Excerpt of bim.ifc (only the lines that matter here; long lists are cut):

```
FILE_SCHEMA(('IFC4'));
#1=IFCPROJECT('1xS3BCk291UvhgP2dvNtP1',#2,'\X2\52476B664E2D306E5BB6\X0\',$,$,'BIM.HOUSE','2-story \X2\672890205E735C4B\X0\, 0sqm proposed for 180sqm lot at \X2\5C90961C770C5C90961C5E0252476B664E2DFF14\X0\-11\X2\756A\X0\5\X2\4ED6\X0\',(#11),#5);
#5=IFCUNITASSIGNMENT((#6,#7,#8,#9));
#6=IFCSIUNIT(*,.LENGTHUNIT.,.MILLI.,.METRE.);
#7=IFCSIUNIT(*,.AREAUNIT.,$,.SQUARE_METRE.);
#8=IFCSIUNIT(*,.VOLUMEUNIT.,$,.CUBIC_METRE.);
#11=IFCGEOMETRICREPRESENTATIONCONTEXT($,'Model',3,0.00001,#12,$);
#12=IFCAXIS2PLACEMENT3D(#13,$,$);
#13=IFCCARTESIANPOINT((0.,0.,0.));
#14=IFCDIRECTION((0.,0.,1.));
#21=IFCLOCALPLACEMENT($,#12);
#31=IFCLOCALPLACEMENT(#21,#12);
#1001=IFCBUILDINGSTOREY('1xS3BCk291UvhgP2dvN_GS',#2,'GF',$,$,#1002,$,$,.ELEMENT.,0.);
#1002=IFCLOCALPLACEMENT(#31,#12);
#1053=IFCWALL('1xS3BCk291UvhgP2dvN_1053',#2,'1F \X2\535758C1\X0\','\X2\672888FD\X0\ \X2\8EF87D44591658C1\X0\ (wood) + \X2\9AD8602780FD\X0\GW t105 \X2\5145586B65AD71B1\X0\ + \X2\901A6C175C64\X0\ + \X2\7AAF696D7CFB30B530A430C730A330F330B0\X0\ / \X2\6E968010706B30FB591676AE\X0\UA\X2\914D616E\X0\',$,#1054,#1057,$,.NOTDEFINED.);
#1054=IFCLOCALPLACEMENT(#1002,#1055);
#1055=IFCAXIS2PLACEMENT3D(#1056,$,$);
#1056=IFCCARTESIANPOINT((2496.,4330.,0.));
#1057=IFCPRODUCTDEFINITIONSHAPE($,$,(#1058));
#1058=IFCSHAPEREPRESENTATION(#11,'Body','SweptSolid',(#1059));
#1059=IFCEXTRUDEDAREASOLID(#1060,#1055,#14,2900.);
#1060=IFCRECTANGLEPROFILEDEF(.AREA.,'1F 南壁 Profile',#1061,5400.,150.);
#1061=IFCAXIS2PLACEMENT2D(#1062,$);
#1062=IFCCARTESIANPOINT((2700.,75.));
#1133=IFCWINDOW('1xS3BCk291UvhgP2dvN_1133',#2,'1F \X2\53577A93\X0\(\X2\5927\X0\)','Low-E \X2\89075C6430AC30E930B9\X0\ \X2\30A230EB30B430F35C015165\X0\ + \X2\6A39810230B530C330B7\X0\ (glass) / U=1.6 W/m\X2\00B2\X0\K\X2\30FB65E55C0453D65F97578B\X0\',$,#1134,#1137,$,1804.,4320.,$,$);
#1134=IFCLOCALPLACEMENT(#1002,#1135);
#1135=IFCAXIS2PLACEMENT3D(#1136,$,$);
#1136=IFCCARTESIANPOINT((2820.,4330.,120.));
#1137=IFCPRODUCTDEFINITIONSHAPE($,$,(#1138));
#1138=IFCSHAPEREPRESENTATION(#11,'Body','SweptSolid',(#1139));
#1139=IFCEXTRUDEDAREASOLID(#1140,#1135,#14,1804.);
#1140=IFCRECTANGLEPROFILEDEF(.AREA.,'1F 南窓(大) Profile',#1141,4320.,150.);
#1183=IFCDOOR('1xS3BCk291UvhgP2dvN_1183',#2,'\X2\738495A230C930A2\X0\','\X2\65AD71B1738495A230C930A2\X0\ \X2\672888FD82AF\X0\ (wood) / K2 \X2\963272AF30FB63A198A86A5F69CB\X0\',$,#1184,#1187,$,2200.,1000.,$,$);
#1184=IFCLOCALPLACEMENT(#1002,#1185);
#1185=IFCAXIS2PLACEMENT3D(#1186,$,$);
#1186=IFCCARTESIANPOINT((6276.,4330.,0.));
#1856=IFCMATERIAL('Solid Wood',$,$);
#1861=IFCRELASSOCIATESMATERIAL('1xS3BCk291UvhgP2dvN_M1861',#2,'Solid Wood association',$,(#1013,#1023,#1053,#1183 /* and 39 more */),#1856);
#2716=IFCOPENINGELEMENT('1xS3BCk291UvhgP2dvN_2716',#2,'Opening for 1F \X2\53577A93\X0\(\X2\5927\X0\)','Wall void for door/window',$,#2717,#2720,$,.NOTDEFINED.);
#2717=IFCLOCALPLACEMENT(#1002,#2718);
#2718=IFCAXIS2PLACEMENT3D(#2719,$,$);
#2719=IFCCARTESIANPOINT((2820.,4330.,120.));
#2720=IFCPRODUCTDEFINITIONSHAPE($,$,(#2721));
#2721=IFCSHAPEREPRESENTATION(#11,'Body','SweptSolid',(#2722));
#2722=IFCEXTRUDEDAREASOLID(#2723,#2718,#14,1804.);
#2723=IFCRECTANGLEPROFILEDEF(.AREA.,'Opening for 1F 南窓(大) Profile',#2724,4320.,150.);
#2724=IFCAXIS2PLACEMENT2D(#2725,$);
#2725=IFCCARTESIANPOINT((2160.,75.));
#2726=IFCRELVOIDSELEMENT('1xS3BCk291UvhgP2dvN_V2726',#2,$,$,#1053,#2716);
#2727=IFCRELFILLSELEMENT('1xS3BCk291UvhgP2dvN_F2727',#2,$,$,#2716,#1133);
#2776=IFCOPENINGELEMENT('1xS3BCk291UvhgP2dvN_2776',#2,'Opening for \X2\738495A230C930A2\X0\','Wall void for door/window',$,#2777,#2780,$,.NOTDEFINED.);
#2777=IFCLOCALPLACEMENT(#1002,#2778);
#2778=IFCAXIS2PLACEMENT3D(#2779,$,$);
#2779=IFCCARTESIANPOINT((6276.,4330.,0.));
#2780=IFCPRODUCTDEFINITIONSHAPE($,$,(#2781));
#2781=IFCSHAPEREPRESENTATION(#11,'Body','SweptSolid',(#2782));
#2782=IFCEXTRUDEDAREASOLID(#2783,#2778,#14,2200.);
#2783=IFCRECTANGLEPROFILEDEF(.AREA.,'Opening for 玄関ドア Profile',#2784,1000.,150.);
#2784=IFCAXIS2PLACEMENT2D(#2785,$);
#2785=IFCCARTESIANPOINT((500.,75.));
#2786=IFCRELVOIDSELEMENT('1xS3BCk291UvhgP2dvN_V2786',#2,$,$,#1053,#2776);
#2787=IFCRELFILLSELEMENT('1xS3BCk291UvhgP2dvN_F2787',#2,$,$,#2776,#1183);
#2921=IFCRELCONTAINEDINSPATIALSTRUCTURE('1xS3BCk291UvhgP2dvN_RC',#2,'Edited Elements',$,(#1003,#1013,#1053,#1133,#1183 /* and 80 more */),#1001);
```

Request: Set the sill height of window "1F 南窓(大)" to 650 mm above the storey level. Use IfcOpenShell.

```python
import numpy as np
import ifcopenshell
import ifcopenshell.api.geometry
import ifcopenshell.geom
import ifcopenshell.util.element
import ifcopenshell.util.placement
import ifcopenshell.util.shape
import ifcopenshell.util.unit

model = ifcopenshell.open("bim.ifc")
unit_scale = ifcopenshell.util.unit.calculate_unit_scale(model)

window = model.by_id(1133)
opening = window.FillsVoids[0].RelatingOpeningElement
storey = ifcopenshell.util.element.get_container(window, ifc_class="IfcBuildingStorey")
level = ifcopenshell.util.placement.get_local_placement(storey.ObjectPlacement)[2, 3]

# The opening's origin need not be at the sill, so measure its lowest point.
shape = ifcopenshell.geom.create_shape(ifcopenshell.geom.settings(), opening)
bottom = ifcopenshell.util.shape.get_shape_bottom_elevation(shape, shape.geometry) / unit_scale
dz = level + 650.0 - bottom

shift = np.array([0.0, 0.0, dz])
# The window is not placed relative to its opening, so move both.
for product in (opening, window):
    matrix = ifcopenshell.util.placement.get_local_placement(product.ObjectPlacement)
    matrix[:3, 3] += shift
    ifcopenshell.api.geometry.edit_object_placement(model, product=product, matrix=matrix, is_si=False)

print(f"moved by {dz * unit_scale:+.3f} m")

model.write("bim_edited.ifc")
```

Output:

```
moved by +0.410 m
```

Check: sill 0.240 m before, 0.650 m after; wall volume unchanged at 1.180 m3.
